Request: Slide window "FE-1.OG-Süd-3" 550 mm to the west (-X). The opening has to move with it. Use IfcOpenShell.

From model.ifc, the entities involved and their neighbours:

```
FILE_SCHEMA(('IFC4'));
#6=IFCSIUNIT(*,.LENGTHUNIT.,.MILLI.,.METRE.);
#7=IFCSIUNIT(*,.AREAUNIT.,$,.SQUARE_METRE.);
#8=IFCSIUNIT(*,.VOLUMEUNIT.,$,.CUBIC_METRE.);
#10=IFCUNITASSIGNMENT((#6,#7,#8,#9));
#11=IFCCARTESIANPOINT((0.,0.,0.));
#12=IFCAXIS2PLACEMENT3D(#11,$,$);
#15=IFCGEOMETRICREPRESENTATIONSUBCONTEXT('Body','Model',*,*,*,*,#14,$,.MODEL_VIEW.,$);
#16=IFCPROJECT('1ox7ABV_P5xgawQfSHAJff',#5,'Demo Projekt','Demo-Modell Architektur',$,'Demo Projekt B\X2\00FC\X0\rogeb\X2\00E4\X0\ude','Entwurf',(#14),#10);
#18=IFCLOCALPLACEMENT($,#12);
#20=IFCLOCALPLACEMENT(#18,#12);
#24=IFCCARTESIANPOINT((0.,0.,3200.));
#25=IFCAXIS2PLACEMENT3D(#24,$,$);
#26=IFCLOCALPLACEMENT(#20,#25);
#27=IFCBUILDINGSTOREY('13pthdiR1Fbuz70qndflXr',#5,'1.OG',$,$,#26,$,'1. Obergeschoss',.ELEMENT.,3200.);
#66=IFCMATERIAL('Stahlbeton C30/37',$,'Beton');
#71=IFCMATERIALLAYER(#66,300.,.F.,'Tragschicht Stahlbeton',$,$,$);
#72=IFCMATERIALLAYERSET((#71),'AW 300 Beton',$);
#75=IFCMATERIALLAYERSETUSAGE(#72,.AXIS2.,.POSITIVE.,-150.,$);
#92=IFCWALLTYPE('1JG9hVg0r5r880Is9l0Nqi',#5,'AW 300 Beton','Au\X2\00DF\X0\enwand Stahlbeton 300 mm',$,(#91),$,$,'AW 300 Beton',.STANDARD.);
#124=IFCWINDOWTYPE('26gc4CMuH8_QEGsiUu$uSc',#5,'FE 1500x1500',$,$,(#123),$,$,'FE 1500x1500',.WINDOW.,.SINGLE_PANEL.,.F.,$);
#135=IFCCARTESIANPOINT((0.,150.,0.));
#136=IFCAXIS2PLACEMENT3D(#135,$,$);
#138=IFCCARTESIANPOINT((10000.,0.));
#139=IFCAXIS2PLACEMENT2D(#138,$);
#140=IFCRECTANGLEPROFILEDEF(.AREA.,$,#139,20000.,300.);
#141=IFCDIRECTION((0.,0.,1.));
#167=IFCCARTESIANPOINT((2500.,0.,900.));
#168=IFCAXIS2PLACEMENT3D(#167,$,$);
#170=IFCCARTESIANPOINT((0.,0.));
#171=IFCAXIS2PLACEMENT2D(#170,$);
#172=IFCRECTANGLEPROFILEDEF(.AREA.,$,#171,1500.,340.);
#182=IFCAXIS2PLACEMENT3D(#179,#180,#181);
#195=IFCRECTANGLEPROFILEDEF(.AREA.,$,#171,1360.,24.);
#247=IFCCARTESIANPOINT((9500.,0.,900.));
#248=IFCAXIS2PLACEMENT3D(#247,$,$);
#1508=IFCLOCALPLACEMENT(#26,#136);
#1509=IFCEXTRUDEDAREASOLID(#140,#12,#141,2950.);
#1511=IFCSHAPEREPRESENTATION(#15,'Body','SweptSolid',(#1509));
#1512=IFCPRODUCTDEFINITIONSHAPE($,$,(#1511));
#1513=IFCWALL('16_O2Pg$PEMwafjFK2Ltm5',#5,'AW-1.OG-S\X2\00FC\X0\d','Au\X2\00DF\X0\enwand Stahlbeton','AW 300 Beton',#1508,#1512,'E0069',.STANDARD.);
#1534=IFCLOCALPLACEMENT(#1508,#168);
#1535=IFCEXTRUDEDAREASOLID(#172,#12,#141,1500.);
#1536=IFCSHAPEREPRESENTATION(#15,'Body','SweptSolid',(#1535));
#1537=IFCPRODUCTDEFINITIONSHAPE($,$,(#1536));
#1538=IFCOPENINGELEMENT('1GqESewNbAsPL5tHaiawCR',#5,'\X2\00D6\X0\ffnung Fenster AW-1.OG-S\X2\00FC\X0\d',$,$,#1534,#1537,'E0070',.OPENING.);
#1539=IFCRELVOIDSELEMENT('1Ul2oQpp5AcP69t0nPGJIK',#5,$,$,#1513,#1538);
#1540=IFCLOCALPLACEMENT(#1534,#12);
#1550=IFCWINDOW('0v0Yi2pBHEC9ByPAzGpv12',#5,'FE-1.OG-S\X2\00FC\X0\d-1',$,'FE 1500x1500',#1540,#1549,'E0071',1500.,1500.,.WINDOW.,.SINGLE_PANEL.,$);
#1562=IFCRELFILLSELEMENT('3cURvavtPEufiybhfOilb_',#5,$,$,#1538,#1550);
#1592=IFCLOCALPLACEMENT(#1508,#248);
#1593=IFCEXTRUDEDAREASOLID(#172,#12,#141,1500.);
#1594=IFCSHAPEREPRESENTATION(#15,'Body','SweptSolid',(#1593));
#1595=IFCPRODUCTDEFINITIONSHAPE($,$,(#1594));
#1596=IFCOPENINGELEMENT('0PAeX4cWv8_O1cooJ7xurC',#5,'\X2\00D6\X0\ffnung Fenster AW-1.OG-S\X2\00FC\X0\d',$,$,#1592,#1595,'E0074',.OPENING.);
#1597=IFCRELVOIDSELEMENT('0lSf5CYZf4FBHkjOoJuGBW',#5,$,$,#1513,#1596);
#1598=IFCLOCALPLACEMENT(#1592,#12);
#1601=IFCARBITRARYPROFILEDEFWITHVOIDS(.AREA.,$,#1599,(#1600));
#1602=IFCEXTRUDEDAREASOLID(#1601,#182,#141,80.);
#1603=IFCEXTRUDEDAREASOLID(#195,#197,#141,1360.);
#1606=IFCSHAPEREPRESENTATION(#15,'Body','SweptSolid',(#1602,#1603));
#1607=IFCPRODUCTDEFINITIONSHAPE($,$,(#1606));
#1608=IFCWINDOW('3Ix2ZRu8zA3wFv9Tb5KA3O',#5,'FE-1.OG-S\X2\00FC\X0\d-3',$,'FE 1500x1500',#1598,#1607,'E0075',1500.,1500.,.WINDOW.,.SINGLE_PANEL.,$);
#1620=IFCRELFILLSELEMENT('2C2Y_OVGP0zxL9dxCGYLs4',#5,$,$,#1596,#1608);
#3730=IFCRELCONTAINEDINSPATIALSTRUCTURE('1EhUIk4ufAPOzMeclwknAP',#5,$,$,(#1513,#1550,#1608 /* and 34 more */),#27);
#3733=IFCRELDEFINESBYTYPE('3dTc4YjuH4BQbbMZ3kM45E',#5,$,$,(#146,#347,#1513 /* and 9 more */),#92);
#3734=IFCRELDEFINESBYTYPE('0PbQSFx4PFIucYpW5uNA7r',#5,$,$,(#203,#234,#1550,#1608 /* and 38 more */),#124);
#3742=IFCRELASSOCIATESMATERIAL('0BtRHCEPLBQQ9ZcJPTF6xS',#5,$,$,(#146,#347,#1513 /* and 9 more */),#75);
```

```python
import ifcopenshell
import ifcopenshell.api.geometry
import ifcopenshell.util.placement
import ifcopenshell.util.unit

model = ifcopenshell.open("model.ifc")
unit_scale = ifcopenshell.util.unit.calculate_unit_scale(model)

window = model.by_guid("3Ix2ZRu8zA3wFv9Tb5KA3O")
opening = window.FillsVoids[0].RelatingOpeningElement
wall = opening.VoidsElements[0].RelatingBuildingElement

wall_matrix = ifcopenshell.util.placement.get_local_placement(wall.ObjectPlacement)
shift = wall_matrix[:3, 0] * -0.55 / unit_scale
before = ifcopenshell.util.placement.get_local_placement(window.ObjectPlacement)[:3, 3].copy()

# The window is placed relative to its opening, so it follows when the opening moves.
matrix = ifcopenshell.util.placement.get_local_placement(opening.ObjectPlacement)
matrix[:3, 3] += shift
ifcopenshell.api.geometry.edit_object_placement(
    model, product=opening, matrix=matrix, is_si=False, should_transform_children=True
)

after = ifcopenshell.util.placement.get_local_placement(window.ObjectPlacement)[:3, 3]
print("window moved by", (after - before).round(3) + 0.0)

model.write("model-out.ifc")
```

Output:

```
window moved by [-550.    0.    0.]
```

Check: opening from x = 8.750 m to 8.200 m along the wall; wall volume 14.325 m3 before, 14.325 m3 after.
